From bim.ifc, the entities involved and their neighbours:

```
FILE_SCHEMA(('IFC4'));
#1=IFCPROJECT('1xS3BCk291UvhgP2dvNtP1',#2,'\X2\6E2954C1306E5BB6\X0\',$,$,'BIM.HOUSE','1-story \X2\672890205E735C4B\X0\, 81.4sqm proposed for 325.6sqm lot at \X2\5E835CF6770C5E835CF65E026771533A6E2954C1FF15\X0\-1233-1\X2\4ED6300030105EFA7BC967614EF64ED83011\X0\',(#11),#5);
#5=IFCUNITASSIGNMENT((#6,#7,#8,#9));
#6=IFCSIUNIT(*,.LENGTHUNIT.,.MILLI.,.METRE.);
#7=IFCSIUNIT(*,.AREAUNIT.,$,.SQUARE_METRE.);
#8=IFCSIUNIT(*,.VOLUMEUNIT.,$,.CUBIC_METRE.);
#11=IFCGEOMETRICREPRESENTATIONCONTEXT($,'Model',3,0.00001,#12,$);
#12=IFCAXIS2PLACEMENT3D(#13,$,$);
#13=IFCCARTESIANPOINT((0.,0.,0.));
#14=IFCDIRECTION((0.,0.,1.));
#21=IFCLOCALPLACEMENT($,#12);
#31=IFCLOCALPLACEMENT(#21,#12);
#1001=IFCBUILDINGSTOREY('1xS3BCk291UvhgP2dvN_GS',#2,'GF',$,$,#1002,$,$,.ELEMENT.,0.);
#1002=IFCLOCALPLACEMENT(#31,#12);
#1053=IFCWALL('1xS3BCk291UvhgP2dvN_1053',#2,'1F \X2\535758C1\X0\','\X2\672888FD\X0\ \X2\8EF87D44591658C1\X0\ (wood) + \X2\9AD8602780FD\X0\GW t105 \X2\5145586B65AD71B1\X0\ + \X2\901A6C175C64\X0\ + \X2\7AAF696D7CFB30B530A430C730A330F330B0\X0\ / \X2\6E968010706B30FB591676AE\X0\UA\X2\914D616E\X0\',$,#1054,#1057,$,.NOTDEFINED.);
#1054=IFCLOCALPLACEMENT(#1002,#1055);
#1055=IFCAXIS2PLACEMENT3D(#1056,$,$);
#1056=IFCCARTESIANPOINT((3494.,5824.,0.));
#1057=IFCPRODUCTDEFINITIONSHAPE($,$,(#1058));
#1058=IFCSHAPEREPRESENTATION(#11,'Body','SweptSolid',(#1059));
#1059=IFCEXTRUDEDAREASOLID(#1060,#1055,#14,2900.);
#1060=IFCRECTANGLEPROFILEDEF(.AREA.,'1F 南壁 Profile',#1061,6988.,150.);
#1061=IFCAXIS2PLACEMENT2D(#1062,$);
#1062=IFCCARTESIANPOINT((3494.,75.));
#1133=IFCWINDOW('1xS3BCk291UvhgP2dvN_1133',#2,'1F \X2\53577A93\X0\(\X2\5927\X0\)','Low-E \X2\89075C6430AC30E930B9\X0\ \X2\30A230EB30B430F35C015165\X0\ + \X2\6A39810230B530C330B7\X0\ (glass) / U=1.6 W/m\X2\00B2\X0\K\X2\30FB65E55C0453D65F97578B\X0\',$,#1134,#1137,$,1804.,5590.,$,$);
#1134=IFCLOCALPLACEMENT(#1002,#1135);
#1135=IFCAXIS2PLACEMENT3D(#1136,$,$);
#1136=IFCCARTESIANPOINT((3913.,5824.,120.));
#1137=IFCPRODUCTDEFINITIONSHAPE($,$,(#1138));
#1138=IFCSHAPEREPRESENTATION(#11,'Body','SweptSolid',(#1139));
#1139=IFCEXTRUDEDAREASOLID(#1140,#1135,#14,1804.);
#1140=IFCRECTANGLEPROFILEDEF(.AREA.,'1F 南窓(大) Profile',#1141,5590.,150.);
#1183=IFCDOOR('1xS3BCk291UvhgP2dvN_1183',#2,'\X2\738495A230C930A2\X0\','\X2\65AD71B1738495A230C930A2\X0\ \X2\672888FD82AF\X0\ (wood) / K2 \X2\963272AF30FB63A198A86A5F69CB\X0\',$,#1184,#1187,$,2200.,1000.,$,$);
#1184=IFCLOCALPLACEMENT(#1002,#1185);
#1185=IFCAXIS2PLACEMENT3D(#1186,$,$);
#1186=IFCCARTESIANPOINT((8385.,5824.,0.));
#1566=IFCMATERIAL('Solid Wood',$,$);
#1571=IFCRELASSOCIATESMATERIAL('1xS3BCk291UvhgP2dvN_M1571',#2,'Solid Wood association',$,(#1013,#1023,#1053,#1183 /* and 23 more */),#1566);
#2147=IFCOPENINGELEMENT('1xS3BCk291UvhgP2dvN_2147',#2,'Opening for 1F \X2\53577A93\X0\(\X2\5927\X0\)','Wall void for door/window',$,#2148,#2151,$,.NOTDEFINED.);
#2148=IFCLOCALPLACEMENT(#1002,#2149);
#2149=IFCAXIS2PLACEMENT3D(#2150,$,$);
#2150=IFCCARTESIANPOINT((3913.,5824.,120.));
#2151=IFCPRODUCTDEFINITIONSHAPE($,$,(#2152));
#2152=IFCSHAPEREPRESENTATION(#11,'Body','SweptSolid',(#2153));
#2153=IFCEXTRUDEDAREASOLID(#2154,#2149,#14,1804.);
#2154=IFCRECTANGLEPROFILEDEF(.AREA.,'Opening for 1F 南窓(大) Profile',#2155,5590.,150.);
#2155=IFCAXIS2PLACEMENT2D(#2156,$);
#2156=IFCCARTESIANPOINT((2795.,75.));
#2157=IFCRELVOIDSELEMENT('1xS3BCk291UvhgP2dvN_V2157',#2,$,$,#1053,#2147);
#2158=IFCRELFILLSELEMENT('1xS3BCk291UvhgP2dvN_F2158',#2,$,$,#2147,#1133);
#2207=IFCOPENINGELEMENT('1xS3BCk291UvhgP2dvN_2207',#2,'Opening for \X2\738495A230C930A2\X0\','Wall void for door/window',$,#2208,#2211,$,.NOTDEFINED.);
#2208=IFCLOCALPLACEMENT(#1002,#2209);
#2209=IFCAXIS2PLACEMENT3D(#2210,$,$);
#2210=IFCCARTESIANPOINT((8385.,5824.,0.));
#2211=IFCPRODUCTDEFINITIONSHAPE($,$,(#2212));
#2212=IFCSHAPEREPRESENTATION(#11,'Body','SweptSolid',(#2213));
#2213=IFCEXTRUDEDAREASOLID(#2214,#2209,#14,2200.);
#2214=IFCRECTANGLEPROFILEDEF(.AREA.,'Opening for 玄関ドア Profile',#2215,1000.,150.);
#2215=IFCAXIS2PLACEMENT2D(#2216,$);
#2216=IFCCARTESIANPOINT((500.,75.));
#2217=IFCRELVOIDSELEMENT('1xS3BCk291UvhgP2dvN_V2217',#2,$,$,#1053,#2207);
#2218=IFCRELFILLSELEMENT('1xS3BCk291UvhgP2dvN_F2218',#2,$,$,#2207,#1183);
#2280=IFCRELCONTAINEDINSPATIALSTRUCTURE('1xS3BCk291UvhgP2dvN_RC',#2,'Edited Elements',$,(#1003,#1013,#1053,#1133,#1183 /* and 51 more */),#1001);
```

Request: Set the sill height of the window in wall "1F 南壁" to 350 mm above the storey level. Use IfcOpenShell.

```python
import numpy as np
import ifcopenshell
import ifcopenshell.api.geometry
import ifcopenshell.geom
import ifcopenshell.util.element
import ifcopenshell.util.placement
import ifcopenshell.util.shape
import ifcopenshell.util.unit

model = ifcopenshell.open("bim.ifc")
unit_scale = ifcopenshell.util.unit.calculate_unit_scale(model)

window = model.by_guid("1xS3BCk291UvhgP2dvN_1133")
opening = window.FillsVoids[0].RelatingOpeningElement
storey = ifcopenshell.util.element.get_container(window, ifc_class="IfcBuildingStorey")
level = ifcopenshell.util.placement.get_local_placement(storey.ObjectPlacement)[2, 3]

# The opening's origin need not be at the sill, so measure its lowest point.
shape = ifcopenshell.geom.create_shape(ifcopenshell.geom.settings(), opening)
bottom = ifcopenshell.util.shape.get_shape_bottom_elevation(shape, shape.geometry) / unit_scale
dz = level + 0.35 / unit_scale - bottom

shift = np.array([0.0, 0.0, dz])
# The window is not placed relative to its opening, so move both.
for product in (opening, window):
    matrix = ifcopenshell.util.placement.get_local_placement(product.ObjectPlacement)
    matrix[:3, 3] += shift
    ifcopenshell.api.geometry.edit_object_placement(model, product=product, matrix=matrix, is_si=False)

print(f"moved by {dz * unit_scale:+.3f} m")

model.write("bim_updated.ifc")
```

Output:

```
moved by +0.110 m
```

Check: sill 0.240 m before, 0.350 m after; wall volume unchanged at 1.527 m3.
